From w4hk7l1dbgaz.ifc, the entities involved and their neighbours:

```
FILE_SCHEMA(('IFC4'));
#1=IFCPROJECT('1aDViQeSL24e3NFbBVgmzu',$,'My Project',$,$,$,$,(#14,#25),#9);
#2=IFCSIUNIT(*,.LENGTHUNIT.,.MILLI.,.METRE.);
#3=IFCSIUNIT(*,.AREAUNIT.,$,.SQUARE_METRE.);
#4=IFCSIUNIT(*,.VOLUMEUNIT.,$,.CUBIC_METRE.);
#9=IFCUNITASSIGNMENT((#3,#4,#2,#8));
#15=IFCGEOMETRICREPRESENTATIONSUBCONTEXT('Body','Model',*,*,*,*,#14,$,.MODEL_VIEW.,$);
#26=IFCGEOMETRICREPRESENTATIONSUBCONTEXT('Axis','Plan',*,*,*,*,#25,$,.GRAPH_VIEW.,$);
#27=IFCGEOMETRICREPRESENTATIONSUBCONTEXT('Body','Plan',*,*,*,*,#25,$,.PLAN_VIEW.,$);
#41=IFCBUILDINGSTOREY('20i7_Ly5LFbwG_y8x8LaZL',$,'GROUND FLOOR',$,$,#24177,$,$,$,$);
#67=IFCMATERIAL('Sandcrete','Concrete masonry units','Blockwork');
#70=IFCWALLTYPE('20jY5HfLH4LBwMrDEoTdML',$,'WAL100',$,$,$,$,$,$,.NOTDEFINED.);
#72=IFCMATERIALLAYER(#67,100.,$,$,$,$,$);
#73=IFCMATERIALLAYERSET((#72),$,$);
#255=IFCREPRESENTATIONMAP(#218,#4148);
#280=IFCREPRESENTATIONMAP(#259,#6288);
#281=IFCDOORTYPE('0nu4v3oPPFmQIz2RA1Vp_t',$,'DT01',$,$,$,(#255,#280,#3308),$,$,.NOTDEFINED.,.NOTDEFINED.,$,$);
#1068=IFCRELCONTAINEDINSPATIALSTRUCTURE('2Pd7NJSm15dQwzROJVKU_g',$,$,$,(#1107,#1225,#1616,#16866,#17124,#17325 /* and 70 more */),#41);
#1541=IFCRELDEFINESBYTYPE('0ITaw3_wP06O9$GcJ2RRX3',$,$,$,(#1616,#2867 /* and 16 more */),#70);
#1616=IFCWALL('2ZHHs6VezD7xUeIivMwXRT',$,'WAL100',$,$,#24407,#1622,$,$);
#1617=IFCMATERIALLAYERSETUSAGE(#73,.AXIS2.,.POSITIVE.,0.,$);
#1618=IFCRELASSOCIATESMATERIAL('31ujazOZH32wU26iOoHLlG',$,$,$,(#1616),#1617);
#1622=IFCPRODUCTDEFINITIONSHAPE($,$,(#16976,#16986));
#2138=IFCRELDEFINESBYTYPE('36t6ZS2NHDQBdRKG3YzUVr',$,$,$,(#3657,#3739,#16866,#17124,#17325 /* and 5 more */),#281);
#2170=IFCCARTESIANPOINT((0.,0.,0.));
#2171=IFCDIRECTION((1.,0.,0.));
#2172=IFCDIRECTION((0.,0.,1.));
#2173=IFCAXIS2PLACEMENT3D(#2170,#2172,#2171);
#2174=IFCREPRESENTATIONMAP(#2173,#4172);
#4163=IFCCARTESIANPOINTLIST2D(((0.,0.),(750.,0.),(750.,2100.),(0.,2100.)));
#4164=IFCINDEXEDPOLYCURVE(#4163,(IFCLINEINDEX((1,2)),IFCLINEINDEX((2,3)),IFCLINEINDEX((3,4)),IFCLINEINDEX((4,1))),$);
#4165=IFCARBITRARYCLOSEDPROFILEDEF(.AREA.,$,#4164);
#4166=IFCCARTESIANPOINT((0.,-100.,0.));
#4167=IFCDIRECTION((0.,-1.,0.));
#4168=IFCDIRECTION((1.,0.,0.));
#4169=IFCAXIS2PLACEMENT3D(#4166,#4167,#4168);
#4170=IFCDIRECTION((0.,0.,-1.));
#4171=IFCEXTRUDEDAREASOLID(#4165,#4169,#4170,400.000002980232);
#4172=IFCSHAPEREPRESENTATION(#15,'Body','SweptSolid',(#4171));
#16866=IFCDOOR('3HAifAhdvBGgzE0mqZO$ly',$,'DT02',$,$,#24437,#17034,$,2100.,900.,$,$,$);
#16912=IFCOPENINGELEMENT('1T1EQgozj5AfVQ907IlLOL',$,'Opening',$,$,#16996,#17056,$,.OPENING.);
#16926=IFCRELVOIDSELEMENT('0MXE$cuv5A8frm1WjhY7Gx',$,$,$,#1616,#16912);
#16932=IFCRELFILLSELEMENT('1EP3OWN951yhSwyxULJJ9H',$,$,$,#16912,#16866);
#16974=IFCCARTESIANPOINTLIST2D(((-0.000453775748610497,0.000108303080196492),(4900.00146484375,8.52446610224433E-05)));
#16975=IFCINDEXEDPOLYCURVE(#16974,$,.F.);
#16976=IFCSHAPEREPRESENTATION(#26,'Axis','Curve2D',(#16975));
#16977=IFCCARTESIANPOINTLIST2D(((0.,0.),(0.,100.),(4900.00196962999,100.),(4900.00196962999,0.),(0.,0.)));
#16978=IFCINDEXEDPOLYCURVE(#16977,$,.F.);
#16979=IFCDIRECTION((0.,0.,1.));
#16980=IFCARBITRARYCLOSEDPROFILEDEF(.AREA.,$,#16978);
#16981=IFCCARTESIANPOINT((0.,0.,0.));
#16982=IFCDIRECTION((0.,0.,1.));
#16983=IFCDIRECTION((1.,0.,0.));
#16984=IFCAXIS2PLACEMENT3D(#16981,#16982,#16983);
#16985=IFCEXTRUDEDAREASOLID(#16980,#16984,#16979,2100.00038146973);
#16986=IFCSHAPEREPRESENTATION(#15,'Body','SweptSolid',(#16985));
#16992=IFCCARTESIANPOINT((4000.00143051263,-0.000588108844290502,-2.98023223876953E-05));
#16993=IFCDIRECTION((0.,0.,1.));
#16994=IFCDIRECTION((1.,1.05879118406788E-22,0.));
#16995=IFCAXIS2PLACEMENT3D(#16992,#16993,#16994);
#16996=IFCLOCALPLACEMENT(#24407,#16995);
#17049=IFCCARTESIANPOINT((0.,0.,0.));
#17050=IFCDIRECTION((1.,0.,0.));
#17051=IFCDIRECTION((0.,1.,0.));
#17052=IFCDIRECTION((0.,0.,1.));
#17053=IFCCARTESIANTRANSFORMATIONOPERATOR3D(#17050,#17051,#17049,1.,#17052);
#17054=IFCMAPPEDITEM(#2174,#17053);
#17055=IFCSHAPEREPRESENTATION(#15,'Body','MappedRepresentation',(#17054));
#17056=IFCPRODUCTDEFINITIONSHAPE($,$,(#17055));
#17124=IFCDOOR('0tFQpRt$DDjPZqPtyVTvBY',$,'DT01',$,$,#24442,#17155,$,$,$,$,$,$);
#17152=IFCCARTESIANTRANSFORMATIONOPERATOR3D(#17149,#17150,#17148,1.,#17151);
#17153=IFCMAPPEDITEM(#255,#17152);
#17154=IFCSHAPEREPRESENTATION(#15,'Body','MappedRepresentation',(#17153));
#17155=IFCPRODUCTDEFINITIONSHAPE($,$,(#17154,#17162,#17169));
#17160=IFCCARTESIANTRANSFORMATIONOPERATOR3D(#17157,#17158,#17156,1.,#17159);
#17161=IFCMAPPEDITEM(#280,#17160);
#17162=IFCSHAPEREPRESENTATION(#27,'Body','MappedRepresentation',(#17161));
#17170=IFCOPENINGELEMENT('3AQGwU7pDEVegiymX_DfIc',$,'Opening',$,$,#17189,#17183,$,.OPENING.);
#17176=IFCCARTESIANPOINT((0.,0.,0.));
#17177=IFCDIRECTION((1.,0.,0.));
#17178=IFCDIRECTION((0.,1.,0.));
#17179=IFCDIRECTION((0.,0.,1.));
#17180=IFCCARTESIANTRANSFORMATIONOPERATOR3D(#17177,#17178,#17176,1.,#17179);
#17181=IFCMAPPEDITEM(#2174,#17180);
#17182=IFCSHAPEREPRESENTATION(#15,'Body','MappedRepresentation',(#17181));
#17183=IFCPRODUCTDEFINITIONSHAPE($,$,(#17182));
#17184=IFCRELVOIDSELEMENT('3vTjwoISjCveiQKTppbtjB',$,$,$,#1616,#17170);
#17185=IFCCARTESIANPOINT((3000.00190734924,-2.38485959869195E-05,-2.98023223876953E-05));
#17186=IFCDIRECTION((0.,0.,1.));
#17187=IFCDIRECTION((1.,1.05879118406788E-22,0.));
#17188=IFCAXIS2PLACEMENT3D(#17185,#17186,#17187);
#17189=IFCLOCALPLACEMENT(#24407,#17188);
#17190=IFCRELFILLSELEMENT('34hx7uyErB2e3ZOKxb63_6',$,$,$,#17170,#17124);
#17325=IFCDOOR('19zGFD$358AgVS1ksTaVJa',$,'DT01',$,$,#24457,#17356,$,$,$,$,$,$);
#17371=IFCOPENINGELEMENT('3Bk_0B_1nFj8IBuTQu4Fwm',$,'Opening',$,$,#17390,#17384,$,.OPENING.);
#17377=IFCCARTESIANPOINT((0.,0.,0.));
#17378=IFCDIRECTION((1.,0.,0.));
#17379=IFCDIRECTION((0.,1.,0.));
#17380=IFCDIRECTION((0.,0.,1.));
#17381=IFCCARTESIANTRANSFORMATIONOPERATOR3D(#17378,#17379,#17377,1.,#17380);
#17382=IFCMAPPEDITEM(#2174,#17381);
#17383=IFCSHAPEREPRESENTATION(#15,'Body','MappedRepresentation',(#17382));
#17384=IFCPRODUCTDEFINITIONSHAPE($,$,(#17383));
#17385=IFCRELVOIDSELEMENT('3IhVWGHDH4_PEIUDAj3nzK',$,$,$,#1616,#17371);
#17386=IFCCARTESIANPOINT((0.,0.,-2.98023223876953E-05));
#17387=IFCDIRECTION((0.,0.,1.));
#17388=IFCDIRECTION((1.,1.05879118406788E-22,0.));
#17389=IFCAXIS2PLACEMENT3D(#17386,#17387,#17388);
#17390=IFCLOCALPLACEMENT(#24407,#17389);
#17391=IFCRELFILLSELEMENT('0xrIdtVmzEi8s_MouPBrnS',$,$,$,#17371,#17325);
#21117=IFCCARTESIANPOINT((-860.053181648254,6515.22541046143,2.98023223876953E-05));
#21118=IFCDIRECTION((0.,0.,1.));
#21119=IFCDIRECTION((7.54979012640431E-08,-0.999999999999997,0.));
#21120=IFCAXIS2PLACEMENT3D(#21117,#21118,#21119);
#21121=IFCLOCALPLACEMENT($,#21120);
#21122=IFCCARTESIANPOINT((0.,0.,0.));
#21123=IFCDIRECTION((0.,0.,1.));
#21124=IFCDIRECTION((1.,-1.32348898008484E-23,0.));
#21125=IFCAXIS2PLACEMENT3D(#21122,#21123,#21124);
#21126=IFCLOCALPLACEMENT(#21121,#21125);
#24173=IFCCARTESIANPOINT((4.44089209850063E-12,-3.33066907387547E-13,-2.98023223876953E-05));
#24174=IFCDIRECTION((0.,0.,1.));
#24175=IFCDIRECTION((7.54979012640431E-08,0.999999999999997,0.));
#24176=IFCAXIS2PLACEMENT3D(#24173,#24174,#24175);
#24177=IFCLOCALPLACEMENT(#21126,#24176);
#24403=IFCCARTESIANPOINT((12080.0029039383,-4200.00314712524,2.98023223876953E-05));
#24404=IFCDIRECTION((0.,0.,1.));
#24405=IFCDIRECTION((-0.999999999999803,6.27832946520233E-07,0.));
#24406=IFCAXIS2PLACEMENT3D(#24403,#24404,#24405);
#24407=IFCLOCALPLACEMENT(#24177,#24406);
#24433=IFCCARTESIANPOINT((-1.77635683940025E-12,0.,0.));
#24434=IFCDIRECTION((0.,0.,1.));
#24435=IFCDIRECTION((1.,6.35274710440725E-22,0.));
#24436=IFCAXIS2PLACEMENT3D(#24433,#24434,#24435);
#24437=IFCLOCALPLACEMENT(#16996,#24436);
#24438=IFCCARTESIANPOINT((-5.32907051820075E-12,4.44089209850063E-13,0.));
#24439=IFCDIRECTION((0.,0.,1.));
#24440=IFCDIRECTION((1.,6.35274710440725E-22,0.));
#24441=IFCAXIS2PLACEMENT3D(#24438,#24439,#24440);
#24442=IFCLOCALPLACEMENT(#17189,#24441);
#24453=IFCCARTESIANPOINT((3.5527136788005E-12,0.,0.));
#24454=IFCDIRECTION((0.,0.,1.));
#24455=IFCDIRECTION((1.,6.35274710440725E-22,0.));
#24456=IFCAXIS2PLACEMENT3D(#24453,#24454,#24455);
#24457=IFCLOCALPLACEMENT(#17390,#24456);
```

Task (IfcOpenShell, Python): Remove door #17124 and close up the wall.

```python
import ifcopenshell
import ifcopenshell.api.feature
import ifcopenshell.api.root
import ifcopenshell.geom
import ifcopenshell.util.shape

model = ifcopenshell.open("w4hk7l1dbgaz.ifc")
settings = ifcopenshell.geom.settings()


def volume(element):
    """Net volume in cubic metres, openings subtracted."""
    shape = ifcopenshell.geom.create_shape(settings, element)
    return ifcopenshell.util.shape.get_volume(shape.geometry)


door = model.by_guid("0tFQpRt$DDjPZqPtyVTvBY")
opening = door.FillsVoids[0].RelatingOpeningElement
wall = opening.VoidsElements[0].RelatingBuildingElement
before = volume(wall)

ifcopenshell.api.root.remove_product(model, product=door)
ifcopenshell.api.feature.remove_feature(model, feature=opening)

after = volume(wall)

print(f"wall volume {before:.3f} -> {after:.3f} m3")

model.write("w4hk7l1dbgaz_edited.ifc")
```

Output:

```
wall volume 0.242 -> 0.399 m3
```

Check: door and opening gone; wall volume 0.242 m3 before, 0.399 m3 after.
